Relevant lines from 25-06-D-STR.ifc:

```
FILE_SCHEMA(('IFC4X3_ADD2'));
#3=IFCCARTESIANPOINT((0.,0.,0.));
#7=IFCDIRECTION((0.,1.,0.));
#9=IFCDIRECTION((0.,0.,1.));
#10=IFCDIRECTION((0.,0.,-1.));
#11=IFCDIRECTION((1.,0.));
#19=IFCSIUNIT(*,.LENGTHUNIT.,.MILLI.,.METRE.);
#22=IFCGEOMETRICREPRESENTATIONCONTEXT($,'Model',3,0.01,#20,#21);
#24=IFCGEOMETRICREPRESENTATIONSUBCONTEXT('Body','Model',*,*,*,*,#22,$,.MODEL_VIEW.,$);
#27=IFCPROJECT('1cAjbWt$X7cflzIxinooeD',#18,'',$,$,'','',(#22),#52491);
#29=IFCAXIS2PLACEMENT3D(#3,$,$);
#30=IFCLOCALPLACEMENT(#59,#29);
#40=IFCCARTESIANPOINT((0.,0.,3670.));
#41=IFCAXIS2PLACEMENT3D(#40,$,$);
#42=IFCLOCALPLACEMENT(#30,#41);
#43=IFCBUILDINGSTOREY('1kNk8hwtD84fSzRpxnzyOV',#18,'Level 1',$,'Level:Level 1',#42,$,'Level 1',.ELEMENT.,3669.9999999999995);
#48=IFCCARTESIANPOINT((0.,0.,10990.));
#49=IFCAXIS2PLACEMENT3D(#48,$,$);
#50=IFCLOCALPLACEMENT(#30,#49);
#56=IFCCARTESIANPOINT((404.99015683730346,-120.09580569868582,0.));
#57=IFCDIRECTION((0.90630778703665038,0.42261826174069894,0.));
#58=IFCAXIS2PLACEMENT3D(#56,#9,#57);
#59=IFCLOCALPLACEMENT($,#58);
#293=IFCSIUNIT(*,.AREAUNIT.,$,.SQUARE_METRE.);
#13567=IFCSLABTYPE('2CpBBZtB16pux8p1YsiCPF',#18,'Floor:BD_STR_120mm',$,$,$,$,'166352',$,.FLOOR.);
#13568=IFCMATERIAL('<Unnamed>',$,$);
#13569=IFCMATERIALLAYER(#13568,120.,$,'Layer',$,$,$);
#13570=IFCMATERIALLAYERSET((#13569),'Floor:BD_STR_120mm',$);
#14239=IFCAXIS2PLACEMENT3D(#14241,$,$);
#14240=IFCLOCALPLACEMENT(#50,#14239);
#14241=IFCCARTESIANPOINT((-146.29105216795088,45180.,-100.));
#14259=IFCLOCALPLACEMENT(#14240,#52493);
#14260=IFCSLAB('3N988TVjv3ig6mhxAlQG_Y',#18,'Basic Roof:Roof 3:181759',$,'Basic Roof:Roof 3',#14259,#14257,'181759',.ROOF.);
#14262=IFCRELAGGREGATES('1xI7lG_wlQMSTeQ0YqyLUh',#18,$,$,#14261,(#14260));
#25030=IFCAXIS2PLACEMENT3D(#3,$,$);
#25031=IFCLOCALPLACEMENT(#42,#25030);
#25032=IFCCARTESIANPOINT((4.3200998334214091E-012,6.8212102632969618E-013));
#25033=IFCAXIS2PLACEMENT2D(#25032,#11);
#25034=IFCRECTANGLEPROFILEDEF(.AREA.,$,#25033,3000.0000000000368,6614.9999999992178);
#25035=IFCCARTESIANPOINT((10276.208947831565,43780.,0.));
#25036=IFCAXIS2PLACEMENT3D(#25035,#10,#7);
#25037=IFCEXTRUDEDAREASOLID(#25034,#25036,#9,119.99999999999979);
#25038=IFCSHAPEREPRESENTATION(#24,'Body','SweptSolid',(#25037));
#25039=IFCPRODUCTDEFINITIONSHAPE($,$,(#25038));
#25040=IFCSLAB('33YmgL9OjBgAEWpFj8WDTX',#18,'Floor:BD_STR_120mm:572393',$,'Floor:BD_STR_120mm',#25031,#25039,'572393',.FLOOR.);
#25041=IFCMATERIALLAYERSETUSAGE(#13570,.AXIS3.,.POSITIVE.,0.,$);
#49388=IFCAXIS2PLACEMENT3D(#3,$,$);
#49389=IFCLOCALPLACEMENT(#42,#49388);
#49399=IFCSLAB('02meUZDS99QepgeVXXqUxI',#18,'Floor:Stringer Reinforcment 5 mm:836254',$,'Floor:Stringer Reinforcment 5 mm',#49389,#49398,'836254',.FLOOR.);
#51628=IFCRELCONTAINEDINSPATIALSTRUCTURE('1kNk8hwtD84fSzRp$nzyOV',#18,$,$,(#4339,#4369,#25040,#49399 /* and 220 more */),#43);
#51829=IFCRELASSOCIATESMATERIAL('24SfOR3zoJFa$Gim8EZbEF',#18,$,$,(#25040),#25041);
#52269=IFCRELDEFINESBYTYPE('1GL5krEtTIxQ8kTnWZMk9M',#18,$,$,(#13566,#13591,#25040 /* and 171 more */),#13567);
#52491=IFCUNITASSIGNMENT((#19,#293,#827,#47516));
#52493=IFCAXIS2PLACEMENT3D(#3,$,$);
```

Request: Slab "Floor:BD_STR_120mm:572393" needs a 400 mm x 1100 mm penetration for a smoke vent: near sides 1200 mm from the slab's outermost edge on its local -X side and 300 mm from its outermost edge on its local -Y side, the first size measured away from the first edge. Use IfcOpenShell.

```python
import numpy as np
import ifcopenshell
import ifcopenshell.api.feature
import ifcopenshell.api.geometry
import ifcopenshell.api.root
import ifcopenshell.geom
import ifcopenshell.util.placement
import ifcopenshell.util.representation
import ifcopenshell.util.shape
import ifcopenshell.util.unit

model = ifcopenshell.open("25-06-D-STR.ifc")
unit_scale = ifcopenshell.util.unit.calculate_unit_scale(model)
settings = ifcopenshell.geom.settings()


def volume(element):
    """Net volume in cubic metres, openings subtracted."""
    shape = ifcopenshell.geom.create_shape(settings, element)
    return ifcopenshell.util.shape.get_volume(shape.geometry)


slab = model.by_guid("33YmgL9OjBgAEWpFj8WDTX")
before = volume(slab)

# Extent in the slab's own axes, in metres. The edges named are its -X and -Y sides.
slab_shape = ifcopenshell.geom.create_shape(settings, slab)
vertices = ifcopenshell.util.shape.get_vertices(slab_shape.geometry)
x_min, y_min, bottom = vertices.min(axis=0)
top = vertices[:, 2].max()

opening = ifcopenshell.api.root.create_entity(model, ifc_class="IfcOpeningElement", name="Smoke vent opening", predefined_type="OPENING")
context = ifcopenshell.util.representation.get_context(model, "Model", "Body", "MODEL_VIEW")
width, depth = 0.4, 1.1
outline = [(0.0, 0.0), (width, 0.0), (width, depth), (0.0, depth), (0.0, 0.0)]
# Overshoot both faces by 50 mm so the cut is clean.
shape = ifcopenshell.api.geometry.add_slab_representation(
    model, context=context, depth=top - bottom + 0.1, polyline=outline
)
ifcopenshell.api.geometry.assign_representation(model, product=opening, representation=shape)

matrix = ifcopenshell.util.placement.get_local_placement(slab.ObjectPlacement)
matrix[:, 3] = matrix @ np.append(np.array([x_min + 1.2, y_min + 0.3, bottom - 0.05]) / unit_scale, 1.0)
ifcopenshell.api.geometry.edit_object_placement(model, product=opening, matrix=matrix, is_si=False)
ifcopenshell.api.feature.add_feature(model, feature=opening, element=slab)

after = volume(slab)

print(f"slab volume {before:.3f} -> {after:.3f} m3")

model.write("25-06-D-STR_v2.ifc")
```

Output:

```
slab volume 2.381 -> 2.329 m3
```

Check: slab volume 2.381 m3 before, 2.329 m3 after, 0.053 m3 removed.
